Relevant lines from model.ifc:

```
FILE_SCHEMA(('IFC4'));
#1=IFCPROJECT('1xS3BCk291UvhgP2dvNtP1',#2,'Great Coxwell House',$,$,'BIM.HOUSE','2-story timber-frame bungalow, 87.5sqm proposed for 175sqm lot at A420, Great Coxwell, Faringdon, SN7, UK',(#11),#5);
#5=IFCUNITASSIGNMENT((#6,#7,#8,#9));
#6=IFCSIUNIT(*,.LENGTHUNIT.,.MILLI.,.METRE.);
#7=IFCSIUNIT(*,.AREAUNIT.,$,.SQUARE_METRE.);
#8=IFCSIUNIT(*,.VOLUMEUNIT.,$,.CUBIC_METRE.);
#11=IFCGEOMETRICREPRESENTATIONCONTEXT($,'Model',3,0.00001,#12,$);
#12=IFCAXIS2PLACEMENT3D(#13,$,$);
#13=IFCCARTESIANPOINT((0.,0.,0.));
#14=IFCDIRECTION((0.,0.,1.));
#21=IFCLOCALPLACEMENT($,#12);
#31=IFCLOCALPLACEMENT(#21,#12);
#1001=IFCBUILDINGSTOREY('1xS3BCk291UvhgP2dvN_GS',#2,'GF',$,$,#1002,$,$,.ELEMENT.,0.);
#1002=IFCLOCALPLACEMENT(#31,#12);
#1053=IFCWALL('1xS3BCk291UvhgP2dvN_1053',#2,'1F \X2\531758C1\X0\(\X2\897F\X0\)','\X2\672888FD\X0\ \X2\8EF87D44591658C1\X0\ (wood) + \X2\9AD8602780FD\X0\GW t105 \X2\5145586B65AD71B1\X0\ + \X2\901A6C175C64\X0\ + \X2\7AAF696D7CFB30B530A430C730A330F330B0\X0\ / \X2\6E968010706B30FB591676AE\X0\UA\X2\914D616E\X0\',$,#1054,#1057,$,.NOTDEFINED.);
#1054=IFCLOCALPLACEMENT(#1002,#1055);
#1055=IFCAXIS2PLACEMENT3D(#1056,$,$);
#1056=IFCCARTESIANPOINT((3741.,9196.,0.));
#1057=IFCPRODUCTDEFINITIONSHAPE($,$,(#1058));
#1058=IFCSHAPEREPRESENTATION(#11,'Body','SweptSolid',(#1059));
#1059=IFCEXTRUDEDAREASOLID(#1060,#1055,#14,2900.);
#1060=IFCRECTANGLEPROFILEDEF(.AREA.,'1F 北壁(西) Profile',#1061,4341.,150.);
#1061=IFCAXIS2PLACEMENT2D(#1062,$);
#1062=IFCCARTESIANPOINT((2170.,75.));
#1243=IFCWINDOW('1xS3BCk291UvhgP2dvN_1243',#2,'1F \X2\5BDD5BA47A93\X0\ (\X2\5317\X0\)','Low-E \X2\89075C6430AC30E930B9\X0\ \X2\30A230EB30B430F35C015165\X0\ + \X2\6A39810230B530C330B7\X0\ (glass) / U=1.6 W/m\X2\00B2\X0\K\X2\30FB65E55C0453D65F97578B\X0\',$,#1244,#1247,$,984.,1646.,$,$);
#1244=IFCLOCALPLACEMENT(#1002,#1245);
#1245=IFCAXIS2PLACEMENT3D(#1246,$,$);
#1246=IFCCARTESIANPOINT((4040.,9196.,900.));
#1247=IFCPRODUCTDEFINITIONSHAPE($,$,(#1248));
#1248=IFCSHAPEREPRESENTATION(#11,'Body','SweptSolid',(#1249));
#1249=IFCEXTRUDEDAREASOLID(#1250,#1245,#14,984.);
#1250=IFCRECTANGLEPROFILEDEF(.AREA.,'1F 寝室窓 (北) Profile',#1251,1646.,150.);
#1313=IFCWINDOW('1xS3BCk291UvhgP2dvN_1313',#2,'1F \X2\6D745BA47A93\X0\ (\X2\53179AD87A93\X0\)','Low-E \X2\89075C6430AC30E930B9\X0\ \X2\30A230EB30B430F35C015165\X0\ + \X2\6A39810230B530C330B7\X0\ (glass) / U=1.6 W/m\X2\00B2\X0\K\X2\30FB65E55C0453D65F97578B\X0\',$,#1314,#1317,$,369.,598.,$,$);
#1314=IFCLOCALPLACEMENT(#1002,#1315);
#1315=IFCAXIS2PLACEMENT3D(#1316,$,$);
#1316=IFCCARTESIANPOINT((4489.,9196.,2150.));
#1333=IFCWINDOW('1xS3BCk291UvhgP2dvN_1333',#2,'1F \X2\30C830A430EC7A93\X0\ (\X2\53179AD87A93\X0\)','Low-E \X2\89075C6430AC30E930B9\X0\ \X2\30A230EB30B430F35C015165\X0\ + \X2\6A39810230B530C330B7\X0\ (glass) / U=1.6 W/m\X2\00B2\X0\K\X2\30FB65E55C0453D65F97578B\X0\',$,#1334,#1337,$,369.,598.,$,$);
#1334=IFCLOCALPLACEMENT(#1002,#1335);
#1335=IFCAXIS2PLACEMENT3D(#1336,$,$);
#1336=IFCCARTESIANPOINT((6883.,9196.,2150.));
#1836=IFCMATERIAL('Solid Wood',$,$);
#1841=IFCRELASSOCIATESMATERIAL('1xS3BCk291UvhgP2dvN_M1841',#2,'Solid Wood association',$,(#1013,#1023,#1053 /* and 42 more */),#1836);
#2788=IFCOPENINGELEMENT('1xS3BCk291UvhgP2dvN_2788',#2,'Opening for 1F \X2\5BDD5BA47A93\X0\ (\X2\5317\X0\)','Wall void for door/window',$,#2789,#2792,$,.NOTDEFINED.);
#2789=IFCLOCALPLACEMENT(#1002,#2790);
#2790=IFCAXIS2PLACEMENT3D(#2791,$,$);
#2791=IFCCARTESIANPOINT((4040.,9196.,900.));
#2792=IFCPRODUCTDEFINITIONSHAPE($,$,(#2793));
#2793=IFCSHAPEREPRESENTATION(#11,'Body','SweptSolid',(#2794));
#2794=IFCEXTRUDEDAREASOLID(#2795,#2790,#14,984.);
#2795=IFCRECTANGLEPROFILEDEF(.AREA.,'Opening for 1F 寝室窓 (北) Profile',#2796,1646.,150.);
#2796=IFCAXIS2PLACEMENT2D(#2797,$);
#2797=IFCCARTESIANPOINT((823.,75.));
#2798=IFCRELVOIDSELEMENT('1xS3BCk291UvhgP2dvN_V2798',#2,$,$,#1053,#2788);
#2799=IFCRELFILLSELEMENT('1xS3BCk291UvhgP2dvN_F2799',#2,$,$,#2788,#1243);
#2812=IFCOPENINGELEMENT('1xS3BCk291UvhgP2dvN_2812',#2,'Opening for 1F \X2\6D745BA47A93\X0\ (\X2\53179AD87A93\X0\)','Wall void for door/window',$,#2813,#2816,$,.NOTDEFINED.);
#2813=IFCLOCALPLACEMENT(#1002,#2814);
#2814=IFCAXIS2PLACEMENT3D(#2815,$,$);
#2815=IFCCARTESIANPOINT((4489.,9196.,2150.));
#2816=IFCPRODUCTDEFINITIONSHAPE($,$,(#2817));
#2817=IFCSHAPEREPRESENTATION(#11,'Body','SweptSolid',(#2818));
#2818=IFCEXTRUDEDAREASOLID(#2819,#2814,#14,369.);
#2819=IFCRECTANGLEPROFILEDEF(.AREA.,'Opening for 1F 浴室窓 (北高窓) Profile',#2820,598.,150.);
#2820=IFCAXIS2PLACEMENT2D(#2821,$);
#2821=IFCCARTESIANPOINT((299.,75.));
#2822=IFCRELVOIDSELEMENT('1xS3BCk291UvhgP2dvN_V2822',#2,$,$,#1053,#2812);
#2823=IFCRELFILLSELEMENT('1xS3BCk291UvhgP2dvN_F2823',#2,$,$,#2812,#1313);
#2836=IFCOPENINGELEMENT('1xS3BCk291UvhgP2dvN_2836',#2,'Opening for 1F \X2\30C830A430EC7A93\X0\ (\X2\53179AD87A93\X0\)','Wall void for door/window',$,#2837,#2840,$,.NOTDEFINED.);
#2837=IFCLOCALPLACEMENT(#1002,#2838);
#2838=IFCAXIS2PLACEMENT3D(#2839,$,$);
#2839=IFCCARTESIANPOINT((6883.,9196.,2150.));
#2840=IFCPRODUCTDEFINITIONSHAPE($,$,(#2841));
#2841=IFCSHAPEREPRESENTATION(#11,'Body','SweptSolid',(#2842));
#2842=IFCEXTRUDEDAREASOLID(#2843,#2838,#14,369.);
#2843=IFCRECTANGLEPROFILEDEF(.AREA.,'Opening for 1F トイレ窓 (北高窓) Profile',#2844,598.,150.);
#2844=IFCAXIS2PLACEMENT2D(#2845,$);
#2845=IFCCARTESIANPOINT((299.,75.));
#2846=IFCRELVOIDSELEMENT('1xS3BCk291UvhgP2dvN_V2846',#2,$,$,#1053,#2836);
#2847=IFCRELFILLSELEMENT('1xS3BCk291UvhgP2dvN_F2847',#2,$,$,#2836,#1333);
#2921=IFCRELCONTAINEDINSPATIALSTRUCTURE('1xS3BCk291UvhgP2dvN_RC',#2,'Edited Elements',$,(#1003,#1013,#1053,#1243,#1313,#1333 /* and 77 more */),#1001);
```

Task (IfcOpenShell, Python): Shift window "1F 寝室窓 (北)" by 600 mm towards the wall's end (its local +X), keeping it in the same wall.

```python
import ifcopenshell
import ifcopenshell.api.geometry
import ifcopenshell.util.placement

model = ifcopenshell.open("model.ifc")

window = model.by_id(1243)
opening = window.FillsVoids[0].RelatingOpeningElement
wall = opening.VoidsElements[0].RelatingBuildingElement

wall_matrix = ifcopenshell.util.placement.get_local_placement(wall.ObjectPlacement)
shift = wall_matrix[:3, 0] * 600.0
before = ifcopenshell.util.placement.get_local_placement(window.ObjectPlacement)[:3, 3].copy()

# The window is not placed relative to its opening, so move both.
for product in (opening, window):
    matrix = ifcopenshell.util.placement.get_local_placement(product.ObjectPlacement)
    matrix[:3, 3] += shift
    ifcopenshell.api.geometry.edit_object_placement(model, product=product, matrix=matrix, is_si=False)

after = ifcopenshell.util.placement.get_local_placement(window.ObjectPlacement)[:3, 3]
print("window moved by", (after - before).round(3) + 0.0)

model.write("model-out.ifc")
```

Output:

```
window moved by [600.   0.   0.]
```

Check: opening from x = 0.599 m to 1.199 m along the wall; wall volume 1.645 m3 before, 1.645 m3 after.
